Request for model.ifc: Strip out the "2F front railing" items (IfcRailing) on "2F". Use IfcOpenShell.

First a look at what the model holds.

```python
import ifcopenshell
import ifcopenshell.util.element

model = ifcopenshell.open("model.ifc")
print(model.schema)
storey = next(s for s in model.by_type("IfcBuildingStorey") if s.Name == "2F")
railings = [e for e in ifcopenshell.util.element.get_decomposition(storey) if e.is_a("IfcRailing")]
seen = {}
for e in railings:
    element_type = ifcopenshell.util.element.get_type(e)
    name = element_type.Name if element_type not in (None, e) else None
    seen[name] = seen.get(name, 0) + 1
for name, count in sorted(seen.items(), key=str):
    print(count, "x", name)
```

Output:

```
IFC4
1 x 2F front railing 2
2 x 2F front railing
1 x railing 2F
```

```python
import ifcopenshell
import ifcopenshell.api.root
import ifcopenshell.util.element

model = ifcopenshell.open("model.ifc")

storey = next(s for s in model.by_type("IfcBuildingStorey") if s.Name == "2F")
railings = [e for e in ifcopenshell.util.element.get_decomposition(storey) if e.is_a("IfcRailing")]
targets = [e for e in railings if (t := ifcopenshell.util.element.get_type(e)) not in (None, e) and t.Name == "2F front railing"]

for e in targets:
    ifcopenshell.api.root.remove_product(model, product=e)
print(len(targets), "removed")

model.write("model_edited.ifc")
```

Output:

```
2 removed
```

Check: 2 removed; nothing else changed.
